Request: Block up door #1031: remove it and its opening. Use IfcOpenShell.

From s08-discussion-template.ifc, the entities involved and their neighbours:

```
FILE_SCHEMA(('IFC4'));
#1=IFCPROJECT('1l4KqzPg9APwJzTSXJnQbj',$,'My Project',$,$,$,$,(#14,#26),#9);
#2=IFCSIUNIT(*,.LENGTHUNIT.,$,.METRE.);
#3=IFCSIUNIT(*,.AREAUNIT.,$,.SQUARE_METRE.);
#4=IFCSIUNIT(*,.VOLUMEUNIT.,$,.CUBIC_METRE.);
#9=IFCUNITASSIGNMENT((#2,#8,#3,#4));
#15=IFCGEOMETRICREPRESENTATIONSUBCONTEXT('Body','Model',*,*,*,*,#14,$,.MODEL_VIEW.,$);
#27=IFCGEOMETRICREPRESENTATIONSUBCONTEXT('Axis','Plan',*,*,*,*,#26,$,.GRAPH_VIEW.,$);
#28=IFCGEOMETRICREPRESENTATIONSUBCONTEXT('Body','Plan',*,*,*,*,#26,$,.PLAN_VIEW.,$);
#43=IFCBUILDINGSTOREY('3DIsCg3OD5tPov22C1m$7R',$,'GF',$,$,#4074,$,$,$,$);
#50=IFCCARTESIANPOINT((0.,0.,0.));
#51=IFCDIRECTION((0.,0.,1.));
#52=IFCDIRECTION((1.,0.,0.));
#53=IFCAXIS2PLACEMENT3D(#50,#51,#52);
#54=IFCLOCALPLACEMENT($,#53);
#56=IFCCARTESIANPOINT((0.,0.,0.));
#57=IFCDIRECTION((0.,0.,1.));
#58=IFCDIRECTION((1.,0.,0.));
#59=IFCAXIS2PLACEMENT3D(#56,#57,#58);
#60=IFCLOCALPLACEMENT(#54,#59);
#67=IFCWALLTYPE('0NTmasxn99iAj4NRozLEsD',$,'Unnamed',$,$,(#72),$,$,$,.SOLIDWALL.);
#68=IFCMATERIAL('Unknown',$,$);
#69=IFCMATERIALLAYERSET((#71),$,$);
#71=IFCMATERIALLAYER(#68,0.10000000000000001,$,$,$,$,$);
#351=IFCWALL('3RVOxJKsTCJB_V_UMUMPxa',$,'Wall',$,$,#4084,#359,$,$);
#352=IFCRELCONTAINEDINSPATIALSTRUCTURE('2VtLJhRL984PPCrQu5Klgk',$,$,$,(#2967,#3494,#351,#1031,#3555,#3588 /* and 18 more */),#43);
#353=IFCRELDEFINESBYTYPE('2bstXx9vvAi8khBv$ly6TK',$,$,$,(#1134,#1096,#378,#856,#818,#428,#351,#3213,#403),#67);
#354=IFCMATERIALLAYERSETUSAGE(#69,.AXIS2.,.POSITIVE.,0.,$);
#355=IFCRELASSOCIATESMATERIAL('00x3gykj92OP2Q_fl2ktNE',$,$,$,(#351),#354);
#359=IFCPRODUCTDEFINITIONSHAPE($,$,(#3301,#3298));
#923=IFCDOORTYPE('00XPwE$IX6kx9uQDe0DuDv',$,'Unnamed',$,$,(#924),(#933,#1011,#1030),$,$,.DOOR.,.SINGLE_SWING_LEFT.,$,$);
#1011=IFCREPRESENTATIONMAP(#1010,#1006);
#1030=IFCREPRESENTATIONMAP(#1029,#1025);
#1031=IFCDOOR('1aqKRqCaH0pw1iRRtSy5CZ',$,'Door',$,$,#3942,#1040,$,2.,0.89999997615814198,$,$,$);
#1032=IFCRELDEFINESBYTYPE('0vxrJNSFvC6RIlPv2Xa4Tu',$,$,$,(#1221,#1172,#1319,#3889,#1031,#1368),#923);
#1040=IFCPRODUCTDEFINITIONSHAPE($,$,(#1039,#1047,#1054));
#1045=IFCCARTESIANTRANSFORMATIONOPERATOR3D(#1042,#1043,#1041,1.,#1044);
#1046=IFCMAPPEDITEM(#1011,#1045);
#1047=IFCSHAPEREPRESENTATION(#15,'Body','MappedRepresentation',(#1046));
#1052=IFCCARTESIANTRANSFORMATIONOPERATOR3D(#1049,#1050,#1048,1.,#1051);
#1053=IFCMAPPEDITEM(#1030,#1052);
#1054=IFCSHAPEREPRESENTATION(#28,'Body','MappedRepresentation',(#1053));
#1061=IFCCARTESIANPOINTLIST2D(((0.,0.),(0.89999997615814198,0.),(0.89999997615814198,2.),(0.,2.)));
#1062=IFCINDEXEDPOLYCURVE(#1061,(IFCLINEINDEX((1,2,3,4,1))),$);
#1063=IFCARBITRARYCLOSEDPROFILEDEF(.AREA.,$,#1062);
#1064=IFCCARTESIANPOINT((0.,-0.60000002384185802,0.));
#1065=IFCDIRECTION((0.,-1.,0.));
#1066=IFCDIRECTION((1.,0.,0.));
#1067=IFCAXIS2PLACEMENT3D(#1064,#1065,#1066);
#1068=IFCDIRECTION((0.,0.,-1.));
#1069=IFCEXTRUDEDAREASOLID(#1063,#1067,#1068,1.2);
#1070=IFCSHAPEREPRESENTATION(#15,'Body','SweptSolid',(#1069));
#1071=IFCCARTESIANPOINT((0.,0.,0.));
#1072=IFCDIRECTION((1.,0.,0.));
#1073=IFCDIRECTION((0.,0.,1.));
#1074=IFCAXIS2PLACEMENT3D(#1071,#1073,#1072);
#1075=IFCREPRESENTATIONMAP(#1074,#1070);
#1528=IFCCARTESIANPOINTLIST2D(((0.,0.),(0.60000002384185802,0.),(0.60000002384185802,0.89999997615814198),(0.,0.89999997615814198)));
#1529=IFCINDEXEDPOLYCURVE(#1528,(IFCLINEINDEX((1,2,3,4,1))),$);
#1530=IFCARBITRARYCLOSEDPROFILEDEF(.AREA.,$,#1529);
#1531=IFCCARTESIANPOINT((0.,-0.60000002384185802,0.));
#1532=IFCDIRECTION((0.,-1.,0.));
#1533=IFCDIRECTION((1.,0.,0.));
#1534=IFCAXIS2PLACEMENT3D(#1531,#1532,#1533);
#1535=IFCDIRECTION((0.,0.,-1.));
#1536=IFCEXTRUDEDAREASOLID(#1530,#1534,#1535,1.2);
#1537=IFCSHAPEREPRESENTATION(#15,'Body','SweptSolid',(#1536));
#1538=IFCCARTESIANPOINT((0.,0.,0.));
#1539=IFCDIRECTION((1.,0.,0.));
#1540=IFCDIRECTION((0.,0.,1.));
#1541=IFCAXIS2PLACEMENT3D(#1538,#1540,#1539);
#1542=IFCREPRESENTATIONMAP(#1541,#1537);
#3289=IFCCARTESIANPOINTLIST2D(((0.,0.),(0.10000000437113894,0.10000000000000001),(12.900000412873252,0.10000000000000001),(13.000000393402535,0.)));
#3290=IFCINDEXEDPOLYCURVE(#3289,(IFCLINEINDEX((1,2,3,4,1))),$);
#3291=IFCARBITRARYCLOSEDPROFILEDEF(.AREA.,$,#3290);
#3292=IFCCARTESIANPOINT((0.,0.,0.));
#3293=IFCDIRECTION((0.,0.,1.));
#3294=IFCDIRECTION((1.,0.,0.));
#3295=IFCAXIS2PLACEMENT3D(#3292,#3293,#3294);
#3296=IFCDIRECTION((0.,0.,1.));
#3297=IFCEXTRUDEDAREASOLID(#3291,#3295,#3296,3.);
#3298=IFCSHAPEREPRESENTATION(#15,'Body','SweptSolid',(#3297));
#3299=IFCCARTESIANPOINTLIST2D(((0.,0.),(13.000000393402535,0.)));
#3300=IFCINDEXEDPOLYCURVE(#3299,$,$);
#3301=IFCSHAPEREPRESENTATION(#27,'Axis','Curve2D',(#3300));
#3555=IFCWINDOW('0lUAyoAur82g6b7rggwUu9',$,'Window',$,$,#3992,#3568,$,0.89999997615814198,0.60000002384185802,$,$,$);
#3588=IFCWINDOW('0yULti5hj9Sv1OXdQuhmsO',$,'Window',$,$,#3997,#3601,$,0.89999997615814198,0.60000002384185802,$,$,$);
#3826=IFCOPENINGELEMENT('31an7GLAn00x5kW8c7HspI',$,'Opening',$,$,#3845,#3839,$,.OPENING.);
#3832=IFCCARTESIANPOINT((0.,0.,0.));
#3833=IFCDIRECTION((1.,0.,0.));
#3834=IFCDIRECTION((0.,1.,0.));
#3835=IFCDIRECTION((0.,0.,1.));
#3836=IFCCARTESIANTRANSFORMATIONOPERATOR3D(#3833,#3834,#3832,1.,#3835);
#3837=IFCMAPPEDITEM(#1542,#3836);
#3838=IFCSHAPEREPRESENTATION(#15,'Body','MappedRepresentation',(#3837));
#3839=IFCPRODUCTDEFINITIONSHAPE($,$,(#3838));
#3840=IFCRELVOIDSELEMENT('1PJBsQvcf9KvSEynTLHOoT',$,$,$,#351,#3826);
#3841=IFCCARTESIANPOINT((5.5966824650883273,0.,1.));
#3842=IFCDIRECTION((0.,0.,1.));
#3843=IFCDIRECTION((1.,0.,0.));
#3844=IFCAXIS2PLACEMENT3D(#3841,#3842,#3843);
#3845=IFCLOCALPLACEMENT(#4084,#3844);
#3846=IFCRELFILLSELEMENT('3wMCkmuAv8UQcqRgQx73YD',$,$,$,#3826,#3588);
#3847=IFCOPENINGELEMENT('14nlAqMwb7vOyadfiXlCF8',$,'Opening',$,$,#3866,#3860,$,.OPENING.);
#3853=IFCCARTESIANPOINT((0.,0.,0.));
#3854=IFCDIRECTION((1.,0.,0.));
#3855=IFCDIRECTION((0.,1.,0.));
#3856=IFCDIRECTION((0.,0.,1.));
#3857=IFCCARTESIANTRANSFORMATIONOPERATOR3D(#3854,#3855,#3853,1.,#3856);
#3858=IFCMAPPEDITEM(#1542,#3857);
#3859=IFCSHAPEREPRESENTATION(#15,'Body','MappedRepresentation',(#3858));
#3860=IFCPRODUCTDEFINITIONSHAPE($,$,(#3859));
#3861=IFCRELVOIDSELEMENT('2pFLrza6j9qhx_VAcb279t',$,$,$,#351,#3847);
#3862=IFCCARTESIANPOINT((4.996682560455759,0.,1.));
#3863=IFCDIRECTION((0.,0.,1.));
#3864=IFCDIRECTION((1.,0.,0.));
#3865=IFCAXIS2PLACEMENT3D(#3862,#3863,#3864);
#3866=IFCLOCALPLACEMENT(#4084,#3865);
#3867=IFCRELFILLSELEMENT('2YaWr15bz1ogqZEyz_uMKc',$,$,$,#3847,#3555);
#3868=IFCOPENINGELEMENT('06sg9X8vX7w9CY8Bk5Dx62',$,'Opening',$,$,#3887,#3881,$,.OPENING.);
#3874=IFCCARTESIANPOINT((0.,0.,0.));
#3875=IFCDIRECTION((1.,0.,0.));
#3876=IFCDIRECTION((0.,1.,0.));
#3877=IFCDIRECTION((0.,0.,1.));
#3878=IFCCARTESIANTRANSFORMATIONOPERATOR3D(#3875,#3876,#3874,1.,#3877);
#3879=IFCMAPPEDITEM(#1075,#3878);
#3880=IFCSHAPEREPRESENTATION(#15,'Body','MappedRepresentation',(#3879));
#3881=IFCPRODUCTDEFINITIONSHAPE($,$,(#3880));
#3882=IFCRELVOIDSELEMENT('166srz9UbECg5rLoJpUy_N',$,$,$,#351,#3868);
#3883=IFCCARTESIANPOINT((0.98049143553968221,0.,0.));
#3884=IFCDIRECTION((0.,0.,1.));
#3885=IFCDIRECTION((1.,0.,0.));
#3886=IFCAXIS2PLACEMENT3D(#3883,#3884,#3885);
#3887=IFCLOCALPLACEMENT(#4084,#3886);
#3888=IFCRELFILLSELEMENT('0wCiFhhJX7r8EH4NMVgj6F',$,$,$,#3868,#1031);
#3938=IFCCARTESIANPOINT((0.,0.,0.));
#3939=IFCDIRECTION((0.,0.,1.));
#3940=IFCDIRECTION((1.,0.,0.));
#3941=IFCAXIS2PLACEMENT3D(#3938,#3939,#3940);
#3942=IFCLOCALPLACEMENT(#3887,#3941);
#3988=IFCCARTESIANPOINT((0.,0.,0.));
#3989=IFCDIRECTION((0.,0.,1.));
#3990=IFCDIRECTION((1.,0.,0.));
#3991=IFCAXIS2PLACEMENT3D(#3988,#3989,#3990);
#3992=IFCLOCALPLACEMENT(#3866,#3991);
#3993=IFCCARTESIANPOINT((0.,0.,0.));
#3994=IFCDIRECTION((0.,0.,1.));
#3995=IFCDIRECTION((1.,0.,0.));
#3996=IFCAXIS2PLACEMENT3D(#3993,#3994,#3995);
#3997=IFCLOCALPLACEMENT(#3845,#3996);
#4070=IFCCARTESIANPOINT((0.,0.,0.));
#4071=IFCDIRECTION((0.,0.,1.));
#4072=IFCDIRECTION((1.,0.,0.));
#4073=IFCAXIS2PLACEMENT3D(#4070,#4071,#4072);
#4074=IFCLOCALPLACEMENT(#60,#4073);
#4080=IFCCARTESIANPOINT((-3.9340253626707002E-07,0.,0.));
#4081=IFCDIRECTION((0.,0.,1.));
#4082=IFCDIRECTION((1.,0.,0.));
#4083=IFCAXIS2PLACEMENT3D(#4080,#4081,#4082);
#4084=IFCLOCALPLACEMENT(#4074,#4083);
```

```python
import ifcopenshell
import ifcopenshell.api.feature
import ifcopenshell.api.root
import ifcopenshell.geom
import ifcopenshell.util.shape

model = ifcopenshell.open("s08-discussion-template.ifc")
settings = ifcopenshell.geom.settings()


def volume(element):
    """Net volume in cubic metres, openings subtracted."""
    shape = ifcopenshell.geom.create_shape(settings, element)
    return ifcopenshell.util.shape.get_volume(shape.geometry)


door = model.by_id(1031)
opening = door.FillsVoids[0].RelatingOpeningElement
wall = opening.VoidsElements[0].RelatingBuildingElement
before = volume(wall)

ifcopenshell.api.root.remove_product(model, product=door)
ifcopenshell.api.feature.remove_feature(model, feature=opening)

after = volume(wall)

print(f"wall volume {before:.3f} -> {after:.3f} m3")

model.write("s08-discussion-template_edited.ifc")
```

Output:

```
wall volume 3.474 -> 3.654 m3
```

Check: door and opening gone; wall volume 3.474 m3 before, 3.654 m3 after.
